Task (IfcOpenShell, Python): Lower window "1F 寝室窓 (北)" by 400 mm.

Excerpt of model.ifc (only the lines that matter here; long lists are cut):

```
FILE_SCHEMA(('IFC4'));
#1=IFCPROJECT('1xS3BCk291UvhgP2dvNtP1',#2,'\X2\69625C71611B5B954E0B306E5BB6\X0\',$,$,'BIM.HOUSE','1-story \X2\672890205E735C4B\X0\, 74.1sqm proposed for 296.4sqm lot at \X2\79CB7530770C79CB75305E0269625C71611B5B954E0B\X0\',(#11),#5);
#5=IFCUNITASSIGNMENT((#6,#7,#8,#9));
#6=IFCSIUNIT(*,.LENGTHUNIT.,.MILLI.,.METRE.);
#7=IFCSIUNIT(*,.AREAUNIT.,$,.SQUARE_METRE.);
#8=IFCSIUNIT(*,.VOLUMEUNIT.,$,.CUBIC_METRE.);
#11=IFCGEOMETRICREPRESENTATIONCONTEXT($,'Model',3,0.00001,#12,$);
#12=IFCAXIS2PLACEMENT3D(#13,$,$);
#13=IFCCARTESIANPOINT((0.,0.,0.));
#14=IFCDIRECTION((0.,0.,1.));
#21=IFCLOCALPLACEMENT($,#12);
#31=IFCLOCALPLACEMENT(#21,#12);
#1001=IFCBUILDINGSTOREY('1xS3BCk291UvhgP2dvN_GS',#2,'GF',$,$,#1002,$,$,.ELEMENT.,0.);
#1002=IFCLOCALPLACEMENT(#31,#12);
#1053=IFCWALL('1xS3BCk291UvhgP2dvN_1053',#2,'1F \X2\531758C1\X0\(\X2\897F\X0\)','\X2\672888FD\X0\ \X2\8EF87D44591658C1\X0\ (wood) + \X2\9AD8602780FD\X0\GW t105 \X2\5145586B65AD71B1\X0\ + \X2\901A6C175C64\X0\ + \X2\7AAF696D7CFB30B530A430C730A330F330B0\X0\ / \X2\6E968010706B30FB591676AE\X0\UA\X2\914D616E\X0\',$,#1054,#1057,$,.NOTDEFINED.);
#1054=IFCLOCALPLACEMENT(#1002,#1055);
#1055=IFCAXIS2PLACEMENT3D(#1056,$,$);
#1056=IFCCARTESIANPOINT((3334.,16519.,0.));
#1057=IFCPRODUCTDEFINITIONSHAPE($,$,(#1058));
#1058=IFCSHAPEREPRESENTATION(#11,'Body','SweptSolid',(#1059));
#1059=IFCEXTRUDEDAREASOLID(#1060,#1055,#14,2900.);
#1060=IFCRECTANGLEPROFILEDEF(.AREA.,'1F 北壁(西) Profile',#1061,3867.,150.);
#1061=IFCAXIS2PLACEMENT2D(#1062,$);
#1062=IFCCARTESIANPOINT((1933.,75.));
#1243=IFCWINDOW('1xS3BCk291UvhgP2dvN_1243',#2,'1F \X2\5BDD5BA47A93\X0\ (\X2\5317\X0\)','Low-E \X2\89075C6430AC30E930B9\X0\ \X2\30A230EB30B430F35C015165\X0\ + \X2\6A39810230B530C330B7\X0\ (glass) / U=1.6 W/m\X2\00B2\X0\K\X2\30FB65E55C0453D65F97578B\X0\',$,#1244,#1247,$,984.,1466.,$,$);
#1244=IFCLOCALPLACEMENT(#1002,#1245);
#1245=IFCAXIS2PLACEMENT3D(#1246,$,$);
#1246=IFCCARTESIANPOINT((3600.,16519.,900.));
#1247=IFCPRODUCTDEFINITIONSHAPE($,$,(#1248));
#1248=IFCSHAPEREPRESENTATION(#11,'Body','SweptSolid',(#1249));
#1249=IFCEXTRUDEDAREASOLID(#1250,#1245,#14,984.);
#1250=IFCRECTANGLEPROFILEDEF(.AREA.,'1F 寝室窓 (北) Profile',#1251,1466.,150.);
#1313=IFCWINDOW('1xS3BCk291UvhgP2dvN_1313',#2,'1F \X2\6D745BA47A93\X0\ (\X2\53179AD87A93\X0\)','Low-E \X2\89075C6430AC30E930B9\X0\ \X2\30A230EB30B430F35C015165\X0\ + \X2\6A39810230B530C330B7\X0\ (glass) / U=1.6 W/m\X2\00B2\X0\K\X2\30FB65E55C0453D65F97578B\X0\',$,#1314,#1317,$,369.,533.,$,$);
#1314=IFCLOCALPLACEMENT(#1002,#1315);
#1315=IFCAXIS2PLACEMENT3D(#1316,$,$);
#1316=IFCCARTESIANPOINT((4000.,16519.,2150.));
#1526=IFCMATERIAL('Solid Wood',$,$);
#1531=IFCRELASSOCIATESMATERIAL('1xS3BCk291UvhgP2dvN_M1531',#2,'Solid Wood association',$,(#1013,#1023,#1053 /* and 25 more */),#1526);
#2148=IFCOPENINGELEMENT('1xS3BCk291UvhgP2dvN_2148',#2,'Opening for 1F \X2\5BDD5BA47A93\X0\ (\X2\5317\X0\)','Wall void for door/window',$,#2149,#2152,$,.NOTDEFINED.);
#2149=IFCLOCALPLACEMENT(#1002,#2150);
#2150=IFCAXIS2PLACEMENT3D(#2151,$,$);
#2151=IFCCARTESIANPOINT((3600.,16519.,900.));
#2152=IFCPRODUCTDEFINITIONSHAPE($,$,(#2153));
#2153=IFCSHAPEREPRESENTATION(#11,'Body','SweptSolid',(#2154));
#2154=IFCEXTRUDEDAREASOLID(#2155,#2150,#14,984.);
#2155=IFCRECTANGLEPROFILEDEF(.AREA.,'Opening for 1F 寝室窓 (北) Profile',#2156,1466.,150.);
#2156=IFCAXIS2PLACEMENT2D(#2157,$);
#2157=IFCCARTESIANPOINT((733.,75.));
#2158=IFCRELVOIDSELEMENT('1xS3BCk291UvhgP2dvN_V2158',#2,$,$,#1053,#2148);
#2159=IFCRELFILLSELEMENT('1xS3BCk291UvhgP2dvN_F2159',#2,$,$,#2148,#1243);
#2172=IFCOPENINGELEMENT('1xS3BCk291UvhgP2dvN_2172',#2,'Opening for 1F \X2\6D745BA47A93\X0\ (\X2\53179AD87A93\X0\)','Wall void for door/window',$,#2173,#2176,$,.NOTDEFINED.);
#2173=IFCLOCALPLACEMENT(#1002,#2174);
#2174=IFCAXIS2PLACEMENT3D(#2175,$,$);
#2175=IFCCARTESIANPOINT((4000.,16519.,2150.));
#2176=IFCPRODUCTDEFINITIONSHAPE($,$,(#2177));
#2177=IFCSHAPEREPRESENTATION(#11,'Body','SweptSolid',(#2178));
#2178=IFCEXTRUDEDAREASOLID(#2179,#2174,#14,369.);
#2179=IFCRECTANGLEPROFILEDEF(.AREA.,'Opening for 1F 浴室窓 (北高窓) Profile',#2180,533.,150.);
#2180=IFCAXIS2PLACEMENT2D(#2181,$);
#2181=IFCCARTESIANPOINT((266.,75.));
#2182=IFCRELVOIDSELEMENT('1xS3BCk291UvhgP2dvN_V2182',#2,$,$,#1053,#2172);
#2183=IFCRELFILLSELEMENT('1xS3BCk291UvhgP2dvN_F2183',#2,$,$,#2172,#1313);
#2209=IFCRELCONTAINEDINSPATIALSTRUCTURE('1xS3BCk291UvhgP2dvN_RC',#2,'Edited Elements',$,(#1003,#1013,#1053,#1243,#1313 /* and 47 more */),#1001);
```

```python
import numpy as np
import ifcopenshell
import ifcopenshell.api.geometry
import ifcopenshell.util.placement
import ifcopenshell.util.unit

model = ifcopenshell.open("model.ifc")
unit_scale = ifcopenshell.util.unit.calculate_unit_scale(model)

window = model.by_guid("1xS3BCk291UvhgP2dvN_1243")
opening = window.FillsVoids[0].RelatingOpeningElement
dz = -0.4 / unit_scale

shift = np.array([0.0, 0.0, dz])
# The window is not placed relative to its opening, so move both.
for product in (opening, window):
    matrix = ifcopenshell.util.placement.get_local_placement(product.ObjectPlacement)
    matrix[:3, 3] += shift
    ifcopenshell.api.geometry.edit_object_placement(model, product=product, matrix=matrix, is_si=False)

print(f"moved by {dz * unit_scale:+.3f} m")

model.write("model_v2.ifc")
```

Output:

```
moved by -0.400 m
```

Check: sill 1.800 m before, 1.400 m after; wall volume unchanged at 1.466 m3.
